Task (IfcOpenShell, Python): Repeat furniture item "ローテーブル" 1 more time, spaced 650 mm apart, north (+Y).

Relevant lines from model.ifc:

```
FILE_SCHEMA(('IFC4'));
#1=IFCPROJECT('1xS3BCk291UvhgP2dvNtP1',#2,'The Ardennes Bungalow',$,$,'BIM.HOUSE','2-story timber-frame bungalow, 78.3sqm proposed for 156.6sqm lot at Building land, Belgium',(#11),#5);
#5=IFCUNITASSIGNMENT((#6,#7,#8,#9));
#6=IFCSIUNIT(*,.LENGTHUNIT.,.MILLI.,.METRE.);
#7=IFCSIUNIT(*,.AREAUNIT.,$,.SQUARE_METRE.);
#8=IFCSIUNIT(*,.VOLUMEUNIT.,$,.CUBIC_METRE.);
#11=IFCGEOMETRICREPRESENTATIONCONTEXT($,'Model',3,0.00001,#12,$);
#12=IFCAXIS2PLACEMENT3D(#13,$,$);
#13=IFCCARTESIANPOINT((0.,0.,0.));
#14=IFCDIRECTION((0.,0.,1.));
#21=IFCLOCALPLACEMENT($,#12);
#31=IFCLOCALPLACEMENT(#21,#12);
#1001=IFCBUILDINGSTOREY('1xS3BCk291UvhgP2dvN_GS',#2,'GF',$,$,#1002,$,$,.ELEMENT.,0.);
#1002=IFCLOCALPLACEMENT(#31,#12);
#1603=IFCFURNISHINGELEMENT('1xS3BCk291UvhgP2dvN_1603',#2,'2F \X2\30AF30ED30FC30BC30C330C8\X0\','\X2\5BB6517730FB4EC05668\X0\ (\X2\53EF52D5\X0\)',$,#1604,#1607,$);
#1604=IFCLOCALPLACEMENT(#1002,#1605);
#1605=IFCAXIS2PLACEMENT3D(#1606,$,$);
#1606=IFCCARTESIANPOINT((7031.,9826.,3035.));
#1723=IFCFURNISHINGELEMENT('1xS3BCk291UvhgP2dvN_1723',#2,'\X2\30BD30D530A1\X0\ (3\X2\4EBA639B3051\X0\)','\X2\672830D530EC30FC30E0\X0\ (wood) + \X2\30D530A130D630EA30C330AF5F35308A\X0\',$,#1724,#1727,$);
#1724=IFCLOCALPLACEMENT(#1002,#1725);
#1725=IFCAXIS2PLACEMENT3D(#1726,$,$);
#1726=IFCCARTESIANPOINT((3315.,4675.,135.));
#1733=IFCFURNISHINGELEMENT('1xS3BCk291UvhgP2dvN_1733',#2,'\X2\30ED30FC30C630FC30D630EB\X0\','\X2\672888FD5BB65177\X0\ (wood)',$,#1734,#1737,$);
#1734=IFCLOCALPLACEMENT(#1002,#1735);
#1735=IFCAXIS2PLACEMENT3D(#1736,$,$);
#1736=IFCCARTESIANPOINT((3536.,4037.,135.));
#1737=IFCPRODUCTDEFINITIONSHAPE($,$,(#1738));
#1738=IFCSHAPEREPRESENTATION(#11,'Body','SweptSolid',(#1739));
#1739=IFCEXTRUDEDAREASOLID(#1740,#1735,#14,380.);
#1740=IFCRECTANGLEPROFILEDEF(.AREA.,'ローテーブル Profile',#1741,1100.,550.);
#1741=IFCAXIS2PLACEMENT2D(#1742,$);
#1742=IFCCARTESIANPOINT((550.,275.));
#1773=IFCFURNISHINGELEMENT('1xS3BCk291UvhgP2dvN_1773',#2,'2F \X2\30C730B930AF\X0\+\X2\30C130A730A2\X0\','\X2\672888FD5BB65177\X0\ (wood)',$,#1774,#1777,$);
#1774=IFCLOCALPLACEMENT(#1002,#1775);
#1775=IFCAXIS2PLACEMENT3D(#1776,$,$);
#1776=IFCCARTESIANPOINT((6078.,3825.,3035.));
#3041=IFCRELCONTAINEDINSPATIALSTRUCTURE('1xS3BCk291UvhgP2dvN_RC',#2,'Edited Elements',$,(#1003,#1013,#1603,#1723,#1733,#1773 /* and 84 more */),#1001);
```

```python
import numpy as np
import ifcopenshell
import ifcopenshell.api.geometry
import ifcopenshell.api.root
import ifcopenshell.util.element
import ifcopenshell.util.placement

model = ifcopenshell.open("model.ifc")


def reuse_history(source, copy):
    """copy_class also copies each property set's owner history, people and application; keep the originals."""
    for rel in copy.IsDefinedBy:
        if rel.is_a("IfcRelDefinesByProperties") and (history := rel.RelatingPropertyDefinition.OwnerHistory):
            rel.RelatingPropertyDefinition.OwnerHistory = source.OwnerHistory
            ifcopenshell.util.element.remove_deep2(model, history)


source = model.by_guid("1xS3BCk291UvhgP2dvN_1733")
base = ifcopenshell.util.placement.get_local_placement(source.ObjectPlacement)
step = np.array([0.0, 1.0, 0.0]) * 650.0

for i in range(1, 2):
    copy = ifcopenshell.api.root.copy_class(model, product=source)
    copy.Representation = ifcopenshell.util.element.copy_deep(
        model, source.Representation, exclude=["IfcGeometricRepresentationContext", "IfcRepresentationMap"]
    )
    reuse_history(source, copy)
    matrix = base.copy()
    matrix[:3, 3] += i * step
    print("added at", matrix[:3, 3].round(3) + 0.0)
    ifcopenshell.api.geometry.edit_object_placement(model, product=copy, matrix=matrix, is_si=False)

model.write("model_updated.ifc")
```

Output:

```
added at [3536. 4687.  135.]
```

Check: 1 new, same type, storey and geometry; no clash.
